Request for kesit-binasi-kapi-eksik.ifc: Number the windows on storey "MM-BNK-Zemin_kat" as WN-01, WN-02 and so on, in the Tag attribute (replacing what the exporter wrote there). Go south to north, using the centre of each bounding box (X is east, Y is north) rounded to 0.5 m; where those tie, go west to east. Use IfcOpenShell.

First a look at what the model holds.

```python
import ifcopenshell
import ifcopenshell.util.element
import ifcopenshell.util.placement

model = ifcopenshell.open("kesit-binasi-kapi-eksik.ifc")
print(model.schema)
storey = next(s for s in model.by_type("IfcBuildingStorey") if s.Name == "MM-BNK-Zemin_kat")
windows = [e for e in ifcopenshell.util.element.get_decomposition(storey) if e.is_a("IfcWindow")]
for e in sorted(windows, key=lambda e: e.id()):
    origin = ifcopenshell.util.placement.get_local_placement(e.ObjectPlacement)[:3, 3]
    print(e.id(), e.Tag, e.Name, origin.round(2) + 0.0, sep=" | ")
```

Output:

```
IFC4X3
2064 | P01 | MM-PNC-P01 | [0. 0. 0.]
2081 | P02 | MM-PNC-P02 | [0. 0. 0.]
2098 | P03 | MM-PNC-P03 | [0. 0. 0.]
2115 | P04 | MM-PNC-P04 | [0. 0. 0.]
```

```python
import ifcopenshell
import ifcopenshell.geom
import ifcopenshell.util.element
import ifcopenshell.util.shape

model = ifcopenshell.open("kesit-binasi-kapi-eksik.ifc")
settings = ifcopenshell.geom.settings()
settings.set("use-world-coords", True)


def centre(element):
    shape = ifcopenshell.geom.create_shape(settings, element)
    return ifcopenshell.util.shape.get_bbox_centroid(shape.geometry)


storey = next(s for s in model.by_type("IfcBuildingStorey") if s.Name == "MM-BNK-Zemin_kat")
windows = [e for e in ifcopenshell.util.element.get_decomposition(storey) if e.is_a("IfcWindow")]

# Insertion points can sit at a corner or the storey origin, so sort by the geometry (in metres).
centres = {e: centre(e) for e in windows}
windows.sort(key=lambda e: (round(centres[e][1] / 0.5), centres[e][0]))

for i, e in enumerate(windows, start=1):
    number = f"WN-{i:02d}"
    e.Tag = number
    print(e.id(), number)

model.write("kesit-binasi-kapi-eksik-out.ifc")
```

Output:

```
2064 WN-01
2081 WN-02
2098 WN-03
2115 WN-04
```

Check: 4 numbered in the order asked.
